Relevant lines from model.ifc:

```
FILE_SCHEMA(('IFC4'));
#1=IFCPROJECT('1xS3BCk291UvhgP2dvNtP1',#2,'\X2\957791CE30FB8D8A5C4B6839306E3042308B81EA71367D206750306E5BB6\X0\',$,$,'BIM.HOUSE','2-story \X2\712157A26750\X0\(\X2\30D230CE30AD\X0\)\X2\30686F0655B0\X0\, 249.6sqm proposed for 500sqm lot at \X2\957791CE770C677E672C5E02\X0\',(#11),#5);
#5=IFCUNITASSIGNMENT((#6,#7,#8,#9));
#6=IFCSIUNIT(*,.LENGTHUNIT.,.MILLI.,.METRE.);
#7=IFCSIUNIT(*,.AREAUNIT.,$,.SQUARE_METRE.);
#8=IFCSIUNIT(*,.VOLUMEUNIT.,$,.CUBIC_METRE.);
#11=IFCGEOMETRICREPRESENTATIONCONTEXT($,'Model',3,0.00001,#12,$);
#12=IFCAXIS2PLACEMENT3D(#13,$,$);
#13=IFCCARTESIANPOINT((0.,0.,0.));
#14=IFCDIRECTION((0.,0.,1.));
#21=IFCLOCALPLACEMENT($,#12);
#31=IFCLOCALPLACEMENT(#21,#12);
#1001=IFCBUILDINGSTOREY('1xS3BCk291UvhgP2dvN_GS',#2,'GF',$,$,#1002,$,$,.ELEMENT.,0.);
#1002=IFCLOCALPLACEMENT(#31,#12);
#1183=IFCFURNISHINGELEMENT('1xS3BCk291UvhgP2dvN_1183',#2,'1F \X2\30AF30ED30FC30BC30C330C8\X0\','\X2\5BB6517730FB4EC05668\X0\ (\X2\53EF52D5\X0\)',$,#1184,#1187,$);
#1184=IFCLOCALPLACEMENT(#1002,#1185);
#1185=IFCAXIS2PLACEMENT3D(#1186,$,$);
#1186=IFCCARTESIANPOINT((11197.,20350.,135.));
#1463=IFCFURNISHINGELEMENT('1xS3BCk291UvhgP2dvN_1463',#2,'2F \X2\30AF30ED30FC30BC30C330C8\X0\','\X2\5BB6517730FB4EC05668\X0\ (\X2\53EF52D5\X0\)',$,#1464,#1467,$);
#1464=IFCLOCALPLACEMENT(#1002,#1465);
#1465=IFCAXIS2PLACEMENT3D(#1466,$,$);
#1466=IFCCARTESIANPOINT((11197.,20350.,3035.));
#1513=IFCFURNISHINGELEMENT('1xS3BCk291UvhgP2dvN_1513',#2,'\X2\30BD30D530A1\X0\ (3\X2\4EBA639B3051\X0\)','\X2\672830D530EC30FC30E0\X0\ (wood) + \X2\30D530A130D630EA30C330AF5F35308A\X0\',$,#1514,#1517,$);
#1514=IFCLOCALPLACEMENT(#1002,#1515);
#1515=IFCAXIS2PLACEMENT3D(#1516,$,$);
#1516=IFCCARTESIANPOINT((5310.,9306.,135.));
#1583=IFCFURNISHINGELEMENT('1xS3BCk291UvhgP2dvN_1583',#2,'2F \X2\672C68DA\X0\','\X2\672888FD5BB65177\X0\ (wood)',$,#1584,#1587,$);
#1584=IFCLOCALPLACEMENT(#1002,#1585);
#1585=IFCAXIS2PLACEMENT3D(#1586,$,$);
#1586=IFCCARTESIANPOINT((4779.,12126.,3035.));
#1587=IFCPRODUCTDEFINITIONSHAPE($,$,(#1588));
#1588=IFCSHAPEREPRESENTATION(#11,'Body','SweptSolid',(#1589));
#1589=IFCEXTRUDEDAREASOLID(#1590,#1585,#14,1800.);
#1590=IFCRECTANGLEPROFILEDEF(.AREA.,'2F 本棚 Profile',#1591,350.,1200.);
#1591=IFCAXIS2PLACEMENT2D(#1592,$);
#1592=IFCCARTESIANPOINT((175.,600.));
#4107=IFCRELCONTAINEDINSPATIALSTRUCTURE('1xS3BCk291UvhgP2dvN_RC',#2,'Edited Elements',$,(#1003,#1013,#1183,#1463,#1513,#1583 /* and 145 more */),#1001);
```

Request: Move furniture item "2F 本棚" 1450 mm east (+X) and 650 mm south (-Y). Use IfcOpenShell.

```python
import ifcopenshell
import ifcopenshell.api.geometry
import ifcopenshell.util.placement

model = ifcopenshell.open("model.ifc")

item = model.by_guid("1xS3BCk291UvhgP2dvN_1583")
matrix = ifcopenshell.util.placement.get_local_placement(item.ObjectPlacement)
matrix[0, 3] += 1450.0
matrix[1, 3] -= 650.0
ifcopenshell.api.geometry.edit_object_placement(model, product=item, matrix=matrix, is_si=False)

print(ifcopenshell.util.placement.get_local_placement(item.ObjectPlacement).round(3) + 0.0)

model.write("model-out.ifc")
```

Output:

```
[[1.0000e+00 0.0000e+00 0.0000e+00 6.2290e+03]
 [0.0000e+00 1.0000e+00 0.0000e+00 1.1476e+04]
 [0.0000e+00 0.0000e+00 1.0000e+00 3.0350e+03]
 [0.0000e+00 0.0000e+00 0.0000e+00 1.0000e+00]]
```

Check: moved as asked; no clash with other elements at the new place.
